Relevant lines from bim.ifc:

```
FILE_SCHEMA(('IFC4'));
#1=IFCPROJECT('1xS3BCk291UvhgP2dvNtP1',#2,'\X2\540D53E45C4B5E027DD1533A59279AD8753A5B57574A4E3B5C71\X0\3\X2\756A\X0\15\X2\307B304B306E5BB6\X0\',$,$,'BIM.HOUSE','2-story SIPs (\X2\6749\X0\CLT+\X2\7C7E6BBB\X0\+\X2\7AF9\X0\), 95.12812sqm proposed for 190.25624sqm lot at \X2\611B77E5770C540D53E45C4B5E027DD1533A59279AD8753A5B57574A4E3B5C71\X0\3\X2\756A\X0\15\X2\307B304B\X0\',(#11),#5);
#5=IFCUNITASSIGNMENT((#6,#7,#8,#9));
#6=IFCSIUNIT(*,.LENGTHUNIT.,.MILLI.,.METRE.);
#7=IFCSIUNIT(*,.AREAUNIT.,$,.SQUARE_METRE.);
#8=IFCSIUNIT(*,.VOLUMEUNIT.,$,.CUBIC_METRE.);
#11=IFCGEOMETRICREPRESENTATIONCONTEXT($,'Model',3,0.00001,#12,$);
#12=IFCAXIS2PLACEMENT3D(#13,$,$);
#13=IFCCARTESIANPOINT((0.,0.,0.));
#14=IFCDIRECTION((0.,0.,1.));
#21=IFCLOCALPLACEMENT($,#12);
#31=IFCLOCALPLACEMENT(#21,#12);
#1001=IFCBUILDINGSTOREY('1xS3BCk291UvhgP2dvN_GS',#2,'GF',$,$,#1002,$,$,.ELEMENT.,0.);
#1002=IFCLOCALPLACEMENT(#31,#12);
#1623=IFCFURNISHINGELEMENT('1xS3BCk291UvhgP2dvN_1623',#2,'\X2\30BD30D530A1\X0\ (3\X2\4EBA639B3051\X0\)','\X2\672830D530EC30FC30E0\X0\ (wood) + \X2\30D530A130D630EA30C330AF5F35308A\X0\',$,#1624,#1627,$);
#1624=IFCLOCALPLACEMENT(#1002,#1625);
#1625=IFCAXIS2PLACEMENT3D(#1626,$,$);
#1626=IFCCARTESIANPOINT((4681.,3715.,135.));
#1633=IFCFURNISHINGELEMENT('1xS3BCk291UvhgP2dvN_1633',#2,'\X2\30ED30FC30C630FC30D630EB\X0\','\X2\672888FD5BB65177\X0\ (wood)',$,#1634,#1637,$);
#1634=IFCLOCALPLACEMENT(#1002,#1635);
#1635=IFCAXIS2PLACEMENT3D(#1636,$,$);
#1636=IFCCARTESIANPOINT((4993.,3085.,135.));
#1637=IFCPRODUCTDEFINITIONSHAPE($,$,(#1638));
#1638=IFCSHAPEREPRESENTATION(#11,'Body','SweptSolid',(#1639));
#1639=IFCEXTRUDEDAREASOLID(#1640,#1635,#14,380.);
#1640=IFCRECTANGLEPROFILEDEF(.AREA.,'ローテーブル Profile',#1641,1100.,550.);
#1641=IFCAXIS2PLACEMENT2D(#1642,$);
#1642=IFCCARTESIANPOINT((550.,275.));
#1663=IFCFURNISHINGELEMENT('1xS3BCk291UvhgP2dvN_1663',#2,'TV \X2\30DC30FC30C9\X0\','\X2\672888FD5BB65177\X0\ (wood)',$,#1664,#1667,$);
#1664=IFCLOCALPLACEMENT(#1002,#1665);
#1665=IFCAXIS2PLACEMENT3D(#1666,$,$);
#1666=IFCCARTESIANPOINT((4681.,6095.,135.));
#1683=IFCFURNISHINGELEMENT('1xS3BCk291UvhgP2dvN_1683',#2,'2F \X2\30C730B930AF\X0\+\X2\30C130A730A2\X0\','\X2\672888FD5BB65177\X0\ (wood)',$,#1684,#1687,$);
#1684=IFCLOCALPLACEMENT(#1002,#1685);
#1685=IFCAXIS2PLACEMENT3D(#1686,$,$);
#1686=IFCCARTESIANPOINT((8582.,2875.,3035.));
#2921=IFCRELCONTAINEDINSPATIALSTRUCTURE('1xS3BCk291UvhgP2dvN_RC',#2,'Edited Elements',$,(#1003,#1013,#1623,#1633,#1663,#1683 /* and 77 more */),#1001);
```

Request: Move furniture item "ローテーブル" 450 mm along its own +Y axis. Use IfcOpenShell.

```python
import ifcopenshell
import ifcopenshell.api.geometry
import ifcopenshell.util.placement
import ifcopenshell.util.unit

model = ifcopenshell.open("bim.ifc")
unit_scale = ifcopenshell.util.unit.calculate_unit_scale(model)

item = model.by_guid("1xS3BCk291UvhgP2dvN_1633")
matrix = ifcopenshell.util.placement.get_local_placement(item.ObjectPlacement)
matrix[:3, 3] += matrix[:3, 1] * 0.45 / unit_scale
ifcopenshell.api.geometry.edit_object_placement(model, product=item, matrix=matrix, is_si=False)

print(ifcopenshell.util.placement.get_local_placement(item.ObjectPlacement).round(3) + 0.0)

model.write("bim-out.ifc")
```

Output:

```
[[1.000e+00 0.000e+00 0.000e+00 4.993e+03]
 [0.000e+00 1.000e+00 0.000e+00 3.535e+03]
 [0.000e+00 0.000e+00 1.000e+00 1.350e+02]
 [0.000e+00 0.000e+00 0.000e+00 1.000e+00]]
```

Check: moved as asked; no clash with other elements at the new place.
